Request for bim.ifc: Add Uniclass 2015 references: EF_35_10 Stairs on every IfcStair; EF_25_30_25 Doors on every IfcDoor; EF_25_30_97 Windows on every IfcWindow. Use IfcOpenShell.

First a look at what the model holds.

```python
import ifcopenshell

model = ifcopenshell.open("bim.ifc")
print(model.schema)
print("classifications:", [c.Name for c in model.by_type("IfcClassification")])
for ifc_class in ("IfcDoor", "IfcRoof", "IfcStair", "IfcWall", "IfcWindow"):
    print(ifc_class, len(model.by_type(ifc_class)))
```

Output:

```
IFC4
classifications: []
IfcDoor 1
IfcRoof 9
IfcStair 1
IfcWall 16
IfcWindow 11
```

```python
import ifcopenshell
import ifcopenshell.api.classification

model = ifcopenshell.open("bim.ifc")

system = ifcopenshell.api.classification.add_classification(model, classification="Uniclass 2015")

codes = {
    "IfcStair": ("EF_35_10", "Stairs"),
    "IfcDoor": ("EF_25_30_25", "Doors"),
    "IfcWindow": ("EF_25_30_97", "Windows"),
}
for ifc_class, (code, name) in codes.items():
    products = model.by_type(ifc_class)
    ifcopenshell.api.classification.add_reference(
        model, products=products, classification=system, identification=code, name=name
    )
    print(code, len(products))

model.write("bim_updated.ifc")
```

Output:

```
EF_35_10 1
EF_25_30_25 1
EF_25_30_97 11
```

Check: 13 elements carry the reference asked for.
